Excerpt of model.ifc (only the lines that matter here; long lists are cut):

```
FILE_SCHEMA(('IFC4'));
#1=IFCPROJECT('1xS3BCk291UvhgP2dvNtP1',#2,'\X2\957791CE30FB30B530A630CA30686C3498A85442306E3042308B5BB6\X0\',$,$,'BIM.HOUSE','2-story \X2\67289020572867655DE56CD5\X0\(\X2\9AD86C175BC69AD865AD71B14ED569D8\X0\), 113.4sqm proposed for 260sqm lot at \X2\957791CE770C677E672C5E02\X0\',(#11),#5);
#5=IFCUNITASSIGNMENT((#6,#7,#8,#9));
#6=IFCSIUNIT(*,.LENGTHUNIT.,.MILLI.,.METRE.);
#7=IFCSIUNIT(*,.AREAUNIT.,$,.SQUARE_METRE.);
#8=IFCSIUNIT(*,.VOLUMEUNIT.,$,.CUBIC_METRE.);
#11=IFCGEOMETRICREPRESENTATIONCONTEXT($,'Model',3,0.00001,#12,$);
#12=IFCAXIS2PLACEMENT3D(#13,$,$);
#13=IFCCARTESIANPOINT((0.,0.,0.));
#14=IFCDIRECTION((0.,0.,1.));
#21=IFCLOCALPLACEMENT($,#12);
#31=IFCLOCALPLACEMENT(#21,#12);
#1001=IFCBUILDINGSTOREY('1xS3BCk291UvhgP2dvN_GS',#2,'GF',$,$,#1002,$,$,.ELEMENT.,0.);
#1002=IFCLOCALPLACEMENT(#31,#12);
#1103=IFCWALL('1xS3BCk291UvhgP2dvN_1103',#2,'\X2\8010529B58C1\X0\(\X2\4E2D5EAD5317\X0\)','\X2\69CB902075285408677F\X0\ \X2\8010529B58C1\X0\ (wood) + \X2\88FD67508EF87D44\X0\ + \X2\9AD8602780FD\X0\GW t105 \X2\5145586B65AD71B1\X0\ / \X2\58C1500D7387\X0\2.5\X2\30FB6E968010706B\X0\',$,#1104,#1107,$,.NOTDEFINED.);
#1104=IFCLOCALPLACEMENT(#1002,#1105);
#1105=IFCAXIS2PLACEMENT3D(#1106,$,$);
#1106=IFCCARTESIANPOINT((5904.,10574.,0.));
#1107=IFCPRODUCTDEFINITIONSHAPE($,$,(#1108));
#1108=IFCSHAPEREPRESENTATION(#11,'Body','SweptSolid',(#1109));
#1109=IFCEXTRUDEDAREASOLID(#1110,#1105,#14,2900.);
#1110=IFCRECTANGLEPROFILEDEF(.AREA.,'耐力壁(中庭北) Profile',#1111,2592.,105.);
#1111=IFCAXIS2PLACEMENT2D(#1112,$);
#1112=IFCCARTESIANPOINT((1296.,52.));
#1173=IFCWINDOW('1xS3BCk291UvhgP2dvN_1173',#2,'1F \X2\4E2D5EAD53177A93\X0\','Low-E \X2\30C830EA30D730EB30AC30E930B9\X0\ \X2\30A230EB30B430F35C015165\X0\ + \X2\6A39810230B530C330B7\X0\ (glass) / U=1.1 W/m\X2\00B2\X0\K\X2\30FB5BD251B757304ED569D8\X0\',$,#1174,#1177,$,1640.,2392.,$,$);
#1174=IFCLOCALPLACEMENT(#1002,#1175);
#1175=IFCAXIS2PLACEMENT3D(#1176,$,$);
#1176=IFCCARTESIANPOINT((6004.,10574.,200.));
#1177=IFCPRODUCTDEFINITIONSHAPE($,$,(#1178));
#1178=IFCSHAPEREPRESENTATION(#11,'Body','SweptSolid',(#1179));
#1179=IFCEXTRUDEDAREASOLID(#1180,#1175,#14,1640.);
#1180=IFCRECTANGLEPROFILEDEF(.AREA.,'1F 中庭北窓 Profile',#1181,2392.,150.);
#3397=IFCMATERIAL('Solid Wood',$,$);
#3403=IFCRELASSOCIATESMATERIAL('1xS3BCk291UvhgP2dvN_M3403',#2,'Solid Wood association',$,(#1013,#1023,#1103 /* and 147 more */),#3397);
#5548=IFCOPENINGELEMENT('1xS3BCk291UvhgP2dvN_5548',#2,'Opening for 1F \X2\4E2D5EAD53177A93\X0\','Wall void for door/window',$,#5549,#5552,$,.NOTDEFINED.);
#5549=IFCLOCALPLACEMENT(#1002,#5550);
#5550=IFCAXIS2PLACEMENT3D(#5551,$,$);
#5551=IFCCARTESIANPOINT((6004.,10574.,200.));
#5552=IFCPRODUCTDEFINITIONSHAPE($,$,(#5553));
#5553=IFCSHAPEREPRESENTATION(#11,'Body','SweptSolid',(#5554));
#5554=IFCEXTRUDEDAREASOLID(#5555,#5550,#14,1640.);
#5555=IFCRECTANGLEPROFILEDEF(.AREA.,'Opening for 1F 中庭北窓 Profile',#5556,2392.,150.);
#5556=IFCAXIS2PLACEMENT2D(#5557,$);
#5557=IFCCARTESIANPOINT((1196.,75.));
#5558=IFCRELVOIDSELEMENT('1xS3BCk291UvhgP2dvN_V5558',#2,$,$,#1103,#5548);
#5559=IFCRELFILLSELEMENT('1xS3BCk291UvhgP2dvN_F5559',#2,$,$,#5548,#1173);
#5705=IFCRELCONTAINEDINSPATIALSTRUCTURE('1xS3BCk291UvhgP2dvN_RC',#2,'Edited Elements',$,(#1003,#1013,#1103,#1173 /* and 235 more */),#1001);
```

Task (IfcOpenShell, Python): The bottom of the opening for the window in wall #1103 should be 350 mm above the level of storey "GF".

```python
import numpy as np
import ifcopenshell
import ifcopenshell.api.geometry
import ifcopenshell.geom
import ifcopenshell.util.element
import ifcopenshell.util.placement
import ifcopenshell.util.shape
import ifcopenshell.util.unit

model = ifcopenshell.open("model.ifc")
unit_scale = ifcopenshell.util.unit.calculate_unit_scale(model)

window = model.by_guid("1xS3BCk291UvhgP2dvN_1173")
opening = window.FillsVoids[0].RelatingOpeningElement
storey = ifcopenshell.util.element.get_container(window, ifc_class="IfcBuildingStorey")
level = ifcopenshell.util.placement.get_local_placement(storey.ObjectPlacement)[2, 3]

# The opening's origin need not be at the sill, so measure its lowest point.
shape = ifcopenshell.geom.create_shape(ifcopenshell.geom.settings(), opening)
bottom = ifcopenshell.util.shape.get_shape_bottom_elevation(shape, shape.geometry) / unit_scale
dz = level + 0.35 / unit_scale - bottom

shift = np.array([0.0, 0.0, dz])
# The window is not placed relative to its opening, so move both.
for product in (opening, window):
    matrix = ifcopenshell.util.placement.get_local_placement(product.ObjectPlacement)
    matrix[:3, 3] += shift
    ifcopenshell.api.geometry.edit_object_placement(model, product=product, matrix=matrix, is_si=False)

print(f"moved by {dz * unit_scale:+.3f} m")

model.write("model_edited.ifc")
```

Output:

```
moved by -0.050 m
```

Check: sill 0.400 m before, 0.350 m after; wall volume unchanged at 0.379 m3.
